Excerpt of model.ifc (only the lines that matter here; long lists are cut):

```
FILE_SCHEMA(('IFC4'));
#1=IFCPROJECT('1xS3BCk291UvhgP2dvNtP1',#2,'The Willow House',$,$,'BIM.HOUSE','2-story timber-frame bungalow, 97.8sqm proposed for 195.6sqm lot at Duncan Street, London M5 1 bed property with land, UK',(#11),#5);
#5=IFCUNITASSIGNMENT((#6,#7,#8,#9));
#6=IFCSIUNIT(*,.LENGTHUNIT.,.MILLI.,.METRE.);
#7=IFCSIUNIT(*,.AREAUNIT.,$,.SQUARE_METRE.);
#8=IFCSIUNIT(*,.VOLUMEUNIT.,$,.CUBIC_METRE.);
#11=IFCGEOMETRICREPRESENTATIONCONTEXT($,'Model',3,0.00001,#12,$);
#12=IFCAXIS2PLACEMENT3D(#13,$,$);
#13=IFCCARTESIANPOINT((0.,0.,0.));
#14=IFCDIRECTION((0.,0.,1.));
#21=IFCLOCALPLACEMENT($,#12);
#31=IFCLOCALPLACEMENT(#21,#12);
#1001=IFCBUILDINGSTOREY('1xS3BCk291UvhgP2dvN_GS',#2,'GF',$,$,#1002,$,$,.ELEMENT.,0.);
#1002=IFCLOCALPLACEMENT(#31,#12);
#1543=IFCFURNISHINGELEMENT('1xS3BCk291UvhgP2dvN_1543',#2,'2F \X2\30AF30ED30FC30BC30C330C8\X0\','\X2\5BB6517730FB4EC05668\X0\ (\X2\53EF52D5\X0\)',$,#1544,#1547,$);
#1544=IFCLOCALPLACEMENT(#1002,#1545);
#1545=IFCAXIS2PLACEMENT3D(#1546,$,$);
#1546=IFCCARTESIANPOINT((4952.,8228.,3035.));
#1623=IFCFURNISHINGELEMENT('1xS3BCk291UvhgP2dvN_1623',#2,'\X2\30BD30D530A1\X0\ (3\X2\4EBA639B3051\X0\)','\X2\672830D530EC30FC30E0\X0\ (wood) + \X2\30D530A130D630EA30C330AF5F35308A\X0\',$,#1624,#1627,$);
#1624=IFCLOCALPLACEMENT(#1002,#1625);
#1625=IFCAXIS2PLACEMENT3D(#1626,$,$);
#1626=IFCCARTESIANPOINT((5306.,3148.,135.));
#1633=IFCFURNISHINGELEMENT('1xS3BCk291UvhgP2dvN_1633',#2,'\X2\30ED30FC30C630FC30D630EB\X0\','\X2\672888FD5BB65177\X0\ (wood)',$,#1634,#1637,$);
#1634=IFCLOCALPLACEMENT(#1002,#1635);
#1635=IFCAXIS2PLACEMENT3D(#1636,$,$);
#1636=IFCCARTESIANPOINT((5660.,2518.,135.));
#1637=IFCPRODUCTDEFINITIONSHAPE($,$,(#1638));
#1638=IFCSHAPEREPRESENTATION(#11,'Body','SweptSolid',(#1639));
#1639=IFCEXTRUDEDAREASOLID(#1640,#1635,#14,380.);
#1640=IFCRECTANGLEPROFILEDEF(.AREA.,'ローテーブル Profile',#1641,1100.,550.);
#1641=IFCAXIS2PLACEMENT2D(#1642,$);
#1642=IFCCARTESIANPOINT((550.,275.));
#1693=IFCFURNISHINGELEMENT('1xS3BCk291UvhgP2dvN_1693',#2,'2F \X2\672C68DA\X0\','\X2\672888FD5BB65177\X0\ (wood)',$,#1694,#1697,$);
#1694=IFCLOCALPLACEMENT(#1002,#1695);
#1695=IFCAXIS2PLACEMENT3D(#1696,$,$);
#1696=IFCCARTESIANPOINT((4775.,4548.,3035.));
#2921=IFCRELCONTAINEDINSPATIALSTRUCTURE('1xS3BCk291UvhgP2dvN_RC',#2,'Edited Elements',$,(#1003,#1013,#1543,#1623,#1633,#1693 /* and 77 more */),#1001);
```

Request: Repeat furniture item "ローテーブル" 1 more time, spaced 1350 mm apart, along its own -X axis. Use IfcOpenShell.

```python
import ifcopenshell
import ifcopenshell.api.geometry
import ifcopenshell.api.root
import ifcopenshell.util.element
import ifcopenshell.util.placement
import ifcopenshell.util.unit

model = ifcopenshell.open("model.ifc")
unit_scale = ifcopenshell.util.unit.calculate_unit_scale(model)


def reuse_history(source, copy):
    """copy_class also copies each property set's owner history, people and application; keep the originals."""
    for rel in copy.IsDefinedBy:
        if rel.is_a("IfcRelDefinesByProperties") and (history := rel.RelatingPropertyDefinition.OwnerHistory):
            rel.RelatingPropertyDefinition.OwnerHistory = source.OwnerHistory
            ifcopenshell.util.element.remove_deep2(model, history)


source = model.by_id(1633)
base = ifcopenshell.util.placement.get_local_placement(source.ObjectPlacement)
step = -base[:3, 0] * 1.35 / unit_scale

for i in range(1, 2):
    copy = ifcopenshell.api.root.copy_class(model, product=source)
    copy.Representation = ifcopenshell.util.element.copy_deep(
        model, source.Representation, exclude=["IfcGeometricRepresentationContext", "IfcRepresentationMap"]
    )
    reuse_history(source, copy)
    matrix = base.copy()
    matrix[:3, 3] += i * step
    print("added at", matrix[:3, 3].round(3) + 0.0)
    ifcopenshell.api.geometry.edit_object_placement(model, product=copy, matrix=matrix, is_si=False)

model.write("model_updated.ifc")
```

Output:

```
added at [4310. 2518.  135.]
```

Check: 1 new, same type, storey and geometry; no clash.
